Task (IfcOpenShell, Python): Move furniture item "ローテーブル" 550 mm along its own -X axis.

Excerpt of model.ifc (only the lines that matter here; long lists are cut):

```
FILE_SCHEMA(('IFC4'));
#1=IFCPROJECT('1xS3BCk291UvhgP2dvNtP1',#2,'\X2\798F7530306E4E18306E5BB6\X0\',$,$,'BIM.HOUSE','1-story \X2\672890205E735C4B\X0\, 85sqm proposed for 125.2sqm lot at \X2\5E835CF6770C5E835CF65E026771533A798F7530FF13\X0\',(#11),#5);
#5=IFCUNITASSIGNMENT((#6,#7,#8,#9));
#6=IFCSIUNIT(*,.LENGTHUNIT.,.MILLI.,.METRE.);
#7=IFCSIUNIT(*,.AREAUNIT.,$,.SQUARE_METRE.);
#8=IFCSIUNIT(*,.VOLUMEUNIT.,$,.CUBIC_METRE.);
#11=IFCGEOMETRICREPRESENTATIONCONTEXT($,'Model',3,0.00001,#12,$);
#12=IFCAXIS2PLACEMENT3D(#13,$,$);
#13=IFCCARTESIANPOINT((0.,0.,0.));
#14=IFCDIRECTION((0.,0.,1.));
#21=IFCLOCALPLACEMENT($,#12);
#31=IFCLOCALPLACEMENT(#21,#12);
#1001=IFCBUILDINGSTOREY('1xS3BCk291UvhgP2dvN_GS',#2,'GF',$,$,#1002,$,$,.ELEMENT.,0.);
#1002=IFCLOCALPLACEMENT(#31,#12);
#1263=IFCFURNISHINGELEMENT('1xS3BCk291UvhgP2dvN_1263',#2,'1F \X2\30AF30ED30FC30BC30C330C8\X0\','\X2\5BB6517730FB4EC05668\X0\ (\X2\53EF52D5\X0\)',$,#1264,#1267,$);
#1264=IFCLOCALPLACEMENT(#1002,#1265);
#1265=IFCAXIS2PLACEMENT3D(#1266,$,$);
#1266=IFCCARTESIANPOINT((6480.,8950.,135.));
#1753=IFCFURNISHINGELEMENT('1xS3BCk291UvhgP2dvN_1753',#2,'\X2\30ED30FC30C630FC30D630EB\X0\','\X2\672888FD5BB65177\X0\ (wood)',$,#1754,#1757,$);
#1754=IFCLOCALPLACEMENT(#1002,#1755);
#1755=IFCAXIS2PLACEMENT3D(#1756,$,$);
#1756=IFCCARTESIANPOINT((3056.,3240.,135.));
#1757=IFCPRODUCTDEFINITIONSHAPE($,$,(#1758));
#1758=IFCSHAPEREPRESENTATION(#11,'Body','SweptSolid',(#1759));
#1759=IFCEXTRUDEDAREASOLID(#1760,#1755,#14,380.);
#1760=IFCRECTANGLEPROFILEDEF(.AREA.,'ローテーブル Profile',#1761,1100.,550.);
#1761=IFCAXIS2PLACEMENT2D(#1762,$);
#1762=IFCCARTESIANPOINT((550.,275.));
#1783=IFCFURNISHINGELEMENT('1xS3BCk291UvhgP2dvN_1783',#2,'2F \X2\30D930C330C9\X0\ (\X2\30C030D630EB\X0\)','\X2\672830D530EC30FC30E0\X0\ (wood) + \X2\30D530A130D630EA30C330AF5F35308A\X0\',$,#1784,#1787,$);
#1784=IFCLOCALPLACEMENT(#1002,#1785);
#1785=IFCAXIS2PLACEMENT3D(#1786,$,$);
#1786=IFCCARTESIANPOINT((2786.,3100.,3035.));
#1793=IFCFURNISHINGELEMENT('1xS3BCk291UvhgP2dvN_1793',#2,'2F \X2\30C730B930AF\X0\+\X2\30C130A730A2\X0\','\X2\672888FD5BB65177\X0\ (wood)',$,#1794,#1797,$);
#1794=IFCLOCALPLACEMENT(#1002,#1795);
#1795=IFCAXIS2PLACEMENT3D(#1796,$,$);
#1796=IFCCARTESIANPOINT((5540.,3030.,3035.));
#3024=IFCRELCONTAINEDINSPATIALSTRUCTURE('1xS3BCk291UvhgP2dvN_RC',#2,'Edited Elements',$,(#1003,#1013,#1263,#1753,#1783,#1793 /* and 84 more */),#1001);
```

```python
import ifcopenshell
import ifcopenshell.api.geometry
import ifcopenshell.util.placement
import ifcopenshell.util.unit

model = ifcopenshell.open("model.ifc")
unit_scale = ifcopenshell.util.unit.calculate_unit_scale(model)

item = model.by_id(1753)
matrix = ifcopenshell.util.placement.get_local_placement(item.ObjectPlacement)
matrix[:3, 3] -= matrix[:3, 0] * 0.55 / unit_scale
ifcopenshell.api.geometry.edit_object_placement(model, product=item, matrix=matrix, is_si=False)

print(ifcopenshell.util.placement.get_local_placement(item.ObjectPlacement).round(3) + 0.0)

model.write("model_updated.ifc")
```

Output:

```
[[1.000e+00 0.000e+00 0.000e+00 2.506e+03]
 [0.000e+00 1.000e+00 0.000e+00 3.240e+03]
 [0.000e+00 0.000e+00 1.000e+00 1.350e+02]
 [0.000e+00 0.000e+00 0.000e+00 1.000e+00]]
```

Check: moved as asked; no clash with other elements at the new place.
